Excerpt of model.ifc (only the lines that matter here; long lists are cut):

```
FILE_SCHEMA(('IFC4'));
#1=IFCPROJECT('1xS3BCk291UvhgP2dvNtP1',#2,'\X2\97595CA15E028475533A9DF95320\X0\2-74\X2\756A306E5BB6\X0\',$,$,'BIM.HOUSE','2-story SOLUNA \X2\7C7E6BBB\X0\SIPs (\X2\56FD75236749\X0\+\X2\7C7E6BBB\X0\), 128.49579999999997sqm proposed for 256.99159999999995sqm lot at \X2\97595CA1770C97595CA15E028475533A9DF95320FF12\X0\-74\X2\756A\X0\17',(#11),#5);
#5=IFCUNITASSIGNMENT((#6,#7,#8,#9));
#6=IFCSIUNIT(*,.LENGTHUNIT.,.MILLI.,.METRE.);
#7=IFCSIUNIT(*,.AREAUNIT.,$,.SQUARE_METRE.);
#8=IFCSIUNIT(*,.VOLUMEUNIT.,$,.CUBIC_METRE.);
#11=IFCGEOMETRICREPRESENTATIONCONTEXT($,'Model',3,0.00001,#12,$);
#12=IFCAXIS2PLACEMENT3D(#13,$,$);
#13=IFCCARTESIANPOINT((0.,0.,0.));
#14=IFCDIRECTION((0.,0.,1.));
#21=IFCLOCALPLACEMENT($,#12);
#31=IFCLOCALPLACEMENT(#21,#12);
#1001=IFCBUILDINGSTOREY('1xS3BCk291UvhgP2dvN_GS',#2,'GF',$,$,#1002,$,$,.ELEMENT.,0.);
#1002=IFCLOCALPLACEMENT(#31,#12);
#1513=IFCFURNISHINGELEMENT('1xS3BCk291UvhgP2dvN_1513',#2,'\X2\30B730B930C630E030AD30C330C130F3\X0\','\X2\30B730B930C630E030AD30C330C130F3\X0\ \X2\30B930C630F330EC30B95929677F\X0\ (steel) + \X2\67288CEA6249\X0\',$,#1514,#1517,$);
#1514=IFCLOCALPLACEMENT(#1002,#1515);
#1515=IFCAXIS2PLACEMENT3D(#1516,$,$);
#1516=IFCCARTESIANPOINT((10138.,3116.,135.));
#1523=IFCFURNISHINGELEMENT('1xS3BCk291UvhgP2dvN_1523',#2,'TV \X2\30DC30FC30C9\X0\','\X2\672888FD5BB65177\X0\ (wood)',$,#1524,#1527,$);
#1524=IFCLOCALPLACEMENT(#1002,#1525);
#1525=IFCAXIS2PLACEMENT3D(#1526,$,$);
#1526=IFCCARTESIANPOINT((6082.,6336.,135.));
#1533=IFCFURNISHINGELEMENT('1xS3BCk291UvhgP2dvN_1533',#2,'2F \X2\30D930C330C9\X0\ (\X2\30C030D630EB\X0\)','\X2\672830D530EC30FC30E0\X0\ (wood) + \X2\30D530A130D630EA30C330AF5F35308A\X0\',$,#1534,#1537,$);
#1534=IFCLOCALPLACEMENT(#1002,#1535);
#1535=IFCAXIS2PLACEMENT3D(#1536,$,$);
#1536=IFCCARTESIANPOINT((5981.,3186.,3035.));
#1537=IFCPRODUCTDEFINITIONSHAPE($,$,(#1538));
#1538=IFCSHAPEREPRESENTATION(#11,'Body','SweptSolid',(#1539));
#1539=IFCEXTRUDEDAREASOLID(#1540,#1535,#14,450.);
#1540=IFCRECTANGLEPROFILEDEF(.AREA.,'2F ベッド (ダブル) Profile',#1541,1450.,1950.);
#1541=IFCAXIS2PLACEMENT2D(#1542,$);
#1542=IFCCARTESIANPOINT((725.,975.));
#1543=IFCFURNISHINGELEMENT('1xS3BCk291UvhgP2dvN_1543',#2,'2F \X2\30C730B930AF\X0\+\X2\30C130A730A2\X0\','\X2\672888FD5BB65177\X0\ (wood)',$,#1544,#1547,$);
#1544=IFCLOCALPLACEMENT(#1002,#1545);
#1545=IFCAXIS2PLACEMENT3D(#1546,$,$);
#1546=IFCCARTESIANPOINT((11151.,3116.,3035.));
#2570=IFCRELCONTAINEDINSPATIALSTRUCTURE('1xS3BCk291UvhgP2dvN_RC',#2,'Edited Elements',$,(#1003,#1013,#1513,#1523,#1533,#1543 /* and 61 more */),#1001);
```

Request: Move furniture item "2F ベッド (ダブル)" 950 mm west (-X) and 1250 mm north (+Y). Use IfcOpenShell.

```python
import ifcopenshell
import ifcopenshell.api.geometry
import ifcopenshell.util.placement

model = ifcopenshell.open("model.ifc")

item = model.by_id(1533)
matrix = ifcopenshell.util.placement.get_local_placement(item.ObjectPlacement)
matrix[0, 3] -= 950.0
matrix[1, 3] += 1250.0
ifcopenshell.api.geometry.edit_object_placement(model, product=item, matrix=matrix, is_si=False)

print(ifcopenshell.util.placement.get_local_placement(item.ObjectPlacement).round(3) + 0.0)

model.write("model_updated.ifc")
```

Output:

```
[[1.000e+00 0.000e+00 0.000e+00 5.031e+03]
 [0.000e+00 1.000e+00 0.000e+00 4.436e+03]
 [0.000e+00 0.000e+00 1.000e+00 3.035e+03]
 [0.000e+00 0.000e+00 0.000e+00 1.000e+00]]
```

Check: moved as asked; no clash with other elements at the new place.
